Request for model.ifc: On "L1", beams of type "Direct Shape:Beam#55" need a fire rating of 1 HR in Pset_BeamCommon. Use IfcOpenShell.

First a look at what the model holds.

```python
import ifcopenshell
import ifcopenshell.util.element

model = ifcopenshell.open("model.ifc")
print(model.schema)
storey = next(s for s in model.by_type("IfcBuildingStorey") if s.Name == "L1")
beams = [e for e in ifcopenshell.util.element.get_decomposition(storey) if e.is_a("IfcBeam")]
seen = {}
for e in beams:
    element_type = ifcopenshell.util.element.get_type(e)
    key = (element_type.Name if element_type != e and element_type else None, ifcopenshell.util.element.get_pset(e, "Pset_BeamCommon", "FireRating"))
    seen[key] = seen.get(key, 0) + 1
for (name, value), count in sorted(seen.items(), key=str):
    print(count, "x", name, "|", value)
```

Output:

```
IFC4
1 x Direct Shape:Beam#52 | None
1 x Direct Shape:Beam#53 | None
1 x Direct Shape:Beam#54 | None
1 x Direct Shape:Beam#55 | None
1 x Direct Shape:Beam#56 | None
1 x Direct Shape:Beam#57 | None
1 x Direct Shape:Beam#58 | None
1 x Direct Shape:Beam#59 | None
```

```python
import ifcopenshell
import ifcopenshell.api.pset
import ifcopenshell.util.element

model = ifcopenshell.open("model.ifc")

storey = next(s for s in model.by_type("IfcBuildingStorey") if s.Name == "L1")
beams = [e for e in ifcopenshell.util.element.get_decomposition(storey) if e.is_a("IfcBeam")]

count = 0
for e in beams:
    element_type = ifcopenshell.util.element.get_type(e)
    if element_type in (None, e) or element_type.Name != "Direct Shape:Beam#55":
        continue
    # add_pset returns the element's existing set when there is one.
    pset = ifcopenshell.api.pset.add_pset(model, product=e, name="Pset_BeamCommon")
    ifcopenshell.api.pset.edit_pset(model, pset=pset, properties={"FireRating": "1 HR"})
    count += 1

print(count, "beams updated")

model.write("model_v2.ifc")
```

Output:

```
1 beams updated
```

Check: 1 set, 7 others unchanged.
